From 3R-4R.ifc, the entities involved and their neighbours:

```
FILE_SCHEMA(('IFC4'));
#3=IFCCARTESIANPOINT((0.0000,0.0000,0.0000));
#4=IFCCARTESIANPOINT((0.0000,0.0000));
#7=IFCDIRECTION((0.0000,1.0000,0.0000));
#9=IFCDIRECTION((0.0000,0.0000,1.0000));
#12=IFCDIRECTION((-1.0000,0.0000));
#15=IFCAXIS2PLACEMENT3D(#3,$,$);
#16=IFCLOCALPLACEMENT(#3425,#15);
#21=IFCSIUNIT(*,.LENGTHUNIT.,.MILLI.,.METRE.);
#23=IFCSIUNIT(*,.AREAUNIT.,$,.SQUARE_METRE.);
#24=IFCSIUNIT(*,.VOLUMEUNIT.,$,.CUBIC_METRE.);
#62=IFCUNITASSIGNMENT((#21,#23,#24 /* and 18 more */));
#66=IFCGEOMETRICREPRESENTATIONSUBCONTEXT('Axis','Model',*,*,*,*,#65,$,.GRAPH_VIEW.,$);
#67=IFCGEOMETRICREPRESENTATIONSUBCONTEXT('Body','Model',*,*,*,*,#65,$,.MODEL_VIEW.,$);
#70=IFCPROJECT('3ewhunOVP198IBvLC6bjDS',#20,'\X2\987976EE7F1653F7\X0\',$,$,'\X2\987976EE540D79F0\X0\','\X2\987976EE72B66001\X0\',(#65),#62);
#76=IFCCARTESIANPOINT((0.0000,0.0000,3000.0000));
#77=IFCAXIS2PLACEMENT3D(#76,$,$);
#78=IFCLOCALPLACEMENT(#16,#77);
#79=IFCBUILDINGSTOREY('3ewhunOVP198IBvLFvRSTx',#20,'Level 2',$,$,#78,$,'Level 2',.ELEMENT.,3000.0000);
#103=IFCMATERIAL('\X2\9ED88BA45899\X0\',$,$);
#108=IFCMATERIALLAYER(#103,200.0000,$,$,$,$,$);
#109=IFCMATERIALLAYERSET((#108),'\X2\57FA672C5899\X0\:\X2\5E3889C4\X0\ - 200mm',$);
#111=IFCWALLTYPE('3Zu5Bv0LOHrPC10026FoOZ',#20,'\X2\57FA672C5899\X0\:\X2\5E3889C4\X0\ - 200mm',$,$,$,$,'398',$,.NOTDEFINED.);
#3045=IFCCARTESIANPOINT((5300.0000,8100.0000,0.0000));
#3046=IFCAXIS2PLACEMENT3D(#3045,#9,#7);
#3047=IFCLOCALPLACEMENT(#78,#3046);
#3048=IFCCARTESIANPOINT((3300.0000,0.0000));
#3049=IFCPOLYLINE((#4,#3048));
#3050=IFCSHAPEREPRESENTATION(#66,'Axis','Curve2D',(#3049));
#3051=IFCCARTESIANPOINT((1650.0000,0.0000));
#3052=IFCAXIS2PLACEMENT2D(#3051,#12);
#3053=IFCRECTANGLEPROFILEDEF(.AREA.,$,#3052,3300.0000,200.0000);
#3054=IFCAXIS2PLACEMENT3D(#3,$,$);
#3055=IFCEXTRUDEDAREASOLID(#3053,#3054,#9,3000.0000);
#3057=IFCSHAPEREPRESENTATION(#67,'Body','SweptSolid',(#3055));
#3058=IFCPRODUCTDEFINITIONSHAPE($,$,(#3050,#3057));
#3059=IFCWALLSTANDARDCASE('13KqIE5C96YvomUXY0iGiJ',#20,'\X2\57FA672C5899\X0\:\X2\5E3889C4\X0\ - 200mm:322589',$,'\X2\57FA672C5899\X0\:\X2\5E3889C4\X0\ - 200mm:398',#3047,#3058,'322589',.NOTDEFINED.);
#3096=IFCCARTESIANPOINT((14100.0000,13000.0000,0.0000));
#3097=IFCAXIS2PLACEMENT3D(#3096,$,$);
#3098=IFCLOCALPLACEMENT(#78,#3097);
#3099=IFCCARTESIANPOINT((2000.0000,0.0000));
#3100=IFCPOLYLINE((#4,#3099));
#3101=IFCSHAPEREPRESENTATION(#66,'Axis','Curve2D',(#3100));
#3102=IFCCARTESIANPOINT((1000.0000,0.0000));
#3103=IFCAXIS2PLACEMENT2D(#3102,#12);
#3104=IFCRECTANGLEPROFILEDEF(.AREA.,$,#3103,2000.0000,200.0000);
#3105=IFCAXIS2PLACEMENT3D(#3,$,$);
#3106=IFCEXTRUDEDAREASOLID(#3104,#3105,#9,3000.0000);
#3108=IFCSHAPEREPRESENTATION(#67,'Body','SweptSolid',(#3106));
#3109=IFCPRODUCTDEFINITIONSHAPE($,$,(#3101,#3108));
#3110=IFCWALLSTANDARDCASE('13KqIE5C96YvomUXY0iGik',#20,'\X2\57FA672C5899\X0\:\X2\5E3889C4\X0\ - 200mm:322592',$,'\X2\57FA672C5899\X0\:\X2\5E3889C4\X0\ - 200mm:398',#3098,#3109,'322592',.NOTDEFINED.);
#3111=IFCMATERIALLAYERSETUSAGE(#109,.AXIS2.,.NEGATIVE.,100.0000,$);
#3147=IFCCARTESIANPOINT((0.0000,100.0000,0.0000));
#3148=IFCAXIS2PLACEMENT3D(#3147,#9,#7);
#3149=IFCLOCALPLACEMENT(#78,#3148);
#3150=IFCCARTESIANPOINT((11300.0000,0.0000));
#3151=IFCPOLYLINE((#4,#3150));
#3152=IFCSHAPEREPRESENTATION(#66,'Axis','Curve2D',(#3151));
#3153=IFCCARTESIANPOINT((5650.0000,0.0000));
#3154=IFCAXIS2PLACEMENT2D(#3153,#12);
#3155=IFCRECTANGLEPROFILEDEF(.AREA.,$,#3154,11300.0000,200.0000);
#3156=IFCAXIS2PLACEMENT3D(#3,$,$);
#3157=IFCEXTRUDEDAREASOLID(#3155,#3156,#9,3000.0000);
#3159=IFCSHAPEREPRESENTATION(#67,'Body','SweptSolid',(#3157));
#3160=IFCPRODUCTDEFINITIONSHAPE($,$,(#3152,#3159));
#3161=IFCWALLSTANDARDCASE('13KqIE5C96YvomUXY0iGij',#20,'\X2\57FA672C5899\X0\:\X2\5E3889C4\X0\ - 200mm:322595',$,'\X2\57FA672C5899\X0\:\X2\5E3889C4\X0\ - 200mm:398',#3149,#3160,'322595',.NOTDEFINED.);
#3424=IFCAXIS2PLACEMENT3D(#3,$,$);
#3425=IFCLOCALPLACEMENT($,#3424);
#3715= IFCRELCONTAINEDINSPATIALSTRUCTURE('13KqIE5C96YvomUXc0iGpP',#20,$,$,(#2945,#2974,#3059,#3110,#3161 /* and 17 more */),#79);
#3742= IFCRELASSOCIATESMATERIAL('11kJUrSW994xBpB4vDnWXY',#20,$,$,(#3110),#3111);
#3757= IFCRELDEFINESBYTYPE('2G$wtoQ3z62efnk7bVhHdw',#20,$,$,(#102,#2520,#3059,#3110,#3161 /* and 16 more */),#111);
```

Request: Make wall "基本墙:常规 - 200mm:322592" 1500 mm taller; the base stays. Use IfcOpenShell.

```python
import ifcopenshell
import ifcopenshell.geom
import ifcopenshell.util.representation
import ifcopenshell.util.shape
import ifcopenshell.util.unit

model = ifcopenshell.open("3R-4R.ifc")
unit_scale = ifcopenshell.util.unit.calculate_unit_scale(model)
settings = ifcopenshell.geom.settings()


def volume(element):
    """Net volume in cubic metres, openings subtracted."""
    shape = ifcopenshell.geom.create_shape(settings, element)
    return ifcopenshell.util.shape.get_volume(shape.geometry)


wall = model.by_guid("13KqIE5C96YvomUXY0iGik")
before = volume(wall)

body = ifcopenshell.util.representation.get_representation(wall, "Model", "Body")
solid = body.Items[0]
old_height = solid.Depth
solid.Depth += 1.5 / unit_scale
after = volume(wall)

print(f"height {old_height:g} -> {solid.Depth:g}, volume {before:.3f} -> {after:.3f} m3")

model.write("3R-4R_edited.ifc")
```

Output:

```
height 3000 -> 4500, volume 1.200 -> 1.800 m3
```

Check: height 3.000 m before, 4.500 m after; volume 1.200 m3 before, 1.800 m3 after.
